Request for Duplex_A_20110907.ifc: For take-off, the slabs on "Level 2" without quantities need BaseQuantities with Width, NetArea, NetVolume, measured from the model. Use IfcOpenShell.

First a look at what the model holds.

```python
import ifcopenshell
import ifcopenshell.util.element
import ifcopenshell.util.unit

model = ifcopenshell.open("Duplex_A_20110907.ifc")
print(model.schema)
for unit_type in ("LENGTHUNIT", "AREAUNIT", "VOLUMEUNIT"):
    print(unit_type, ifcopenshell.util.unit.calculate_unit_scale(model, unit_type))
storey = next(s for s in model.by_type("IfcBuildingStorey") if s.Name == "Level 2")
slabs = [e for e in ifcopenshell.util.element.get_decomposition(storey) if e.is_a("IfcSlab")]
for e in sorted(slabs, key=lambda e: e.id()):
    print(e.id(), e.is_a(), e.Name, list(ifcopenshell.util.element.get_psets(e, qtos_only=True)), sep=" | ")
```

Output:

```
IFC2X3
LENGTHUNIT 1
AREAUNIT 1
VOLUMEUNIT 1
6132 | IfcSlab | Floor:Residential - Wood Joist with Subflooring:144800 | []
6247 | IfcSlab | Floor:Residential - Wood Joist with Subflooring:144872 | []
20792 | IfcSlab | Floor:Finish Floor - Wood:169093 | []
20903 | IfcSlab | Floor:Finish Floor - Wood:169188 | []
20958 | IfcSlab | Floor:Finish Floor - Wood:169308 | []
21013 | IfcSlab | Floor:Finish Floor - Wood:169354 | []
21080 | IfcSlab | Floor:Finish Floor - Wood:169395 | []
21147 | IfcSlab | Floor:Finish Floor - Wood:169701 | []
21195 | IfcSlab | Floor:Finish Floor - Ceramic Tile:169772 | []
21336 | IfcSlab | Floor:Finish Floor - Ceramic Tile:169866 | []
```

```python
import ifcopenshell
import ifcopenshell.api.pset
import ifcopenshell.geom
import ifcopenshell.util.element
import ifcopenshell.util.shape
import ifcopenshell.util.unit

model = ifcopenshell.open("Duplex_A_20110907.ifc")
unit_scale = ifcopenshell.util.unit.calculate_unit_scale(model)
area_scale = ifcopenshell.util.unit.calculate_unit_scale(model, "AREAUNIT")
volume_scale = ifcopenshell.util.unit.calculate_unit_scale(model, "VOLUMEUNIT")
settings = ifcopenshell.geom.settings()

storey = next(s for s in model.by_type("IfcBuildingStorey") if s.Name == "Level 2")
slabs = [e for e in ifcopenshell.util.element.get_decomposition(storey) if e.is_a("IfcSlab")]

for e in sorted(slabs, key=lambda e: e.id()):
    if ifcopenshell.util.element.get_psets(e, qtos_only=True, should_inherit=False):
        continue
    # Geometry comes back in metres, in the element's own axes.
    shape = ifcopenshell.geom.create_shape(settings, e)
    values = {
        "Width": ifcopenshell.util.shape.get_z(shape.geometry) / unit_scale,
        "NetArea": ifcopenshell.util.shape.get_footprint_area(shape.geometry) / area_scale,
        "NetVolume": ifcopenshell.util.shape.get_volume(shape.geometry) / volume_scale,
    }
    qto = ifcopenshell.api.pset.add_qto(model, product=e, name="BaseQuantities")
    ifcopenshell.api.pset.edit_qto(model, qto=qto, properties=values)
    print(e.id(), {k: round(v, 3) for k, v in values.items()})

model.write("Duplex_A_20110907_rev.ifc")
```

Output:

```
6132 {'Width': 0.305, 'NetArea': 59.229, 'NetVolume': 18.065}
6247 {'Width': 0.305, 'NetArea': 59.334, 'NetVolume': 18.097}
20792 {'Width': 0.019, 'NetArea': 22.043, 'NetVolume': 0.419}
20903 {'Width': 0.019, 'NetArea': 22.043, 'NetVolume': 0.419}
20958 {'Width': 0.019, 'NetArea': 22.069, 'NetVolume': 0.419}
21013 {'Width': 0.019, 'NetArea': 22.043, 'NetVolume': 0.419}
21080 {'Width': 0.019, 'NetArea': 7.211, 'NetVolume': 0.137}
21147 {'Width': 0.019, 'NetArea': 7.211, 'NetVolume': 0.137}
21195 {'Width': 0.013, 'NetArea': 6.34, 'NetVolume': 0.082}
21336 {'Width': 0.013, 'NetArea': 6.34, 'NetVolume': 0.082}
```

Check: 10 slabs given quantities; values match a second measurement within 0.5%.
